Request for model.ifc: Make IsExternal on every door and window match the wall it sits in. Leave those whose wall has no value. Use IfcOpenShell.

First a look at what the model holds.

```python
import ifcopenshell
import ifcopenshell.util.element

model = ifcopenshell.open("model.ifc")
print(model.schema)
seen = {}
for e in model.by_type("IfcDoor") + model.by_type("IfcWindow"):
    if not e.FillsVoids:
        continue
    host = e.FillsVoids[0].RelatingOpeningElement.VoidsElements[0].RelatingBuildingElement
    own = ifcopenshell.util.element.get_pset(e, f"Pset_{e.is_a()[3:].removesuffix('StandardCase')}Common", "IsExternal")
    wall = ifcopenshell.util.element.get_pset(host, "Pset_WallCommon", "IsExternal")
    seen[e.is_a(), own, wall] = seen.get((e.is_a(), own, wall), 0) + 1
for (cls, own, wall), count in sorted(seen.items(), key=str):
    print(count, cls, "IsExternal:", own, "| host wall:", wall)
```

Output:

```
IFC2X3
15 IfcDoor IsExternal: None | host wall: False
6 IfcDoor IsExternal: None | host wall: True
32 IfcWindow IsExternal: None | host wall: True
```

```python
import ifcopenshell
import ifcopenshell.api.pset
import ifcopenshell.util.element

model = ifcopenshell.open("model.ifc")

count = 0
for ifc_class, pset_name in (("IfcDoor", "Pset_DoorCommon"), ("IfcWindow", "Pset_WindowCommon")):
    for e in model.by_type(ifc_class):
        if not e.FillsVoids:
            continue
        host = e.FillsVoids[0].RelatingOpeningElement.VoidsElements[0].RelatingBuildingElement
        external = ifcopenshell.util.element.get_pset(host, "Pset_WallCommon", "IsExternal")
        if external is None or ifcopenshell.util.element.get_pset(e, pset_name, "IsExternal") == external:
            continue
        pset = ifcopenshell.api.pset.add_pset(model, product=e, name=pset_name)
        ifcopenshell.api.pset.edit_pset(model, pset=pset, properties={"IsExternal": external})
        count += 1

print(count, "updated")

model.write("model-out.ifc")
```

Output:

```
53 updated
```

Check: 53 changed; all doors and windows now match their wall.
